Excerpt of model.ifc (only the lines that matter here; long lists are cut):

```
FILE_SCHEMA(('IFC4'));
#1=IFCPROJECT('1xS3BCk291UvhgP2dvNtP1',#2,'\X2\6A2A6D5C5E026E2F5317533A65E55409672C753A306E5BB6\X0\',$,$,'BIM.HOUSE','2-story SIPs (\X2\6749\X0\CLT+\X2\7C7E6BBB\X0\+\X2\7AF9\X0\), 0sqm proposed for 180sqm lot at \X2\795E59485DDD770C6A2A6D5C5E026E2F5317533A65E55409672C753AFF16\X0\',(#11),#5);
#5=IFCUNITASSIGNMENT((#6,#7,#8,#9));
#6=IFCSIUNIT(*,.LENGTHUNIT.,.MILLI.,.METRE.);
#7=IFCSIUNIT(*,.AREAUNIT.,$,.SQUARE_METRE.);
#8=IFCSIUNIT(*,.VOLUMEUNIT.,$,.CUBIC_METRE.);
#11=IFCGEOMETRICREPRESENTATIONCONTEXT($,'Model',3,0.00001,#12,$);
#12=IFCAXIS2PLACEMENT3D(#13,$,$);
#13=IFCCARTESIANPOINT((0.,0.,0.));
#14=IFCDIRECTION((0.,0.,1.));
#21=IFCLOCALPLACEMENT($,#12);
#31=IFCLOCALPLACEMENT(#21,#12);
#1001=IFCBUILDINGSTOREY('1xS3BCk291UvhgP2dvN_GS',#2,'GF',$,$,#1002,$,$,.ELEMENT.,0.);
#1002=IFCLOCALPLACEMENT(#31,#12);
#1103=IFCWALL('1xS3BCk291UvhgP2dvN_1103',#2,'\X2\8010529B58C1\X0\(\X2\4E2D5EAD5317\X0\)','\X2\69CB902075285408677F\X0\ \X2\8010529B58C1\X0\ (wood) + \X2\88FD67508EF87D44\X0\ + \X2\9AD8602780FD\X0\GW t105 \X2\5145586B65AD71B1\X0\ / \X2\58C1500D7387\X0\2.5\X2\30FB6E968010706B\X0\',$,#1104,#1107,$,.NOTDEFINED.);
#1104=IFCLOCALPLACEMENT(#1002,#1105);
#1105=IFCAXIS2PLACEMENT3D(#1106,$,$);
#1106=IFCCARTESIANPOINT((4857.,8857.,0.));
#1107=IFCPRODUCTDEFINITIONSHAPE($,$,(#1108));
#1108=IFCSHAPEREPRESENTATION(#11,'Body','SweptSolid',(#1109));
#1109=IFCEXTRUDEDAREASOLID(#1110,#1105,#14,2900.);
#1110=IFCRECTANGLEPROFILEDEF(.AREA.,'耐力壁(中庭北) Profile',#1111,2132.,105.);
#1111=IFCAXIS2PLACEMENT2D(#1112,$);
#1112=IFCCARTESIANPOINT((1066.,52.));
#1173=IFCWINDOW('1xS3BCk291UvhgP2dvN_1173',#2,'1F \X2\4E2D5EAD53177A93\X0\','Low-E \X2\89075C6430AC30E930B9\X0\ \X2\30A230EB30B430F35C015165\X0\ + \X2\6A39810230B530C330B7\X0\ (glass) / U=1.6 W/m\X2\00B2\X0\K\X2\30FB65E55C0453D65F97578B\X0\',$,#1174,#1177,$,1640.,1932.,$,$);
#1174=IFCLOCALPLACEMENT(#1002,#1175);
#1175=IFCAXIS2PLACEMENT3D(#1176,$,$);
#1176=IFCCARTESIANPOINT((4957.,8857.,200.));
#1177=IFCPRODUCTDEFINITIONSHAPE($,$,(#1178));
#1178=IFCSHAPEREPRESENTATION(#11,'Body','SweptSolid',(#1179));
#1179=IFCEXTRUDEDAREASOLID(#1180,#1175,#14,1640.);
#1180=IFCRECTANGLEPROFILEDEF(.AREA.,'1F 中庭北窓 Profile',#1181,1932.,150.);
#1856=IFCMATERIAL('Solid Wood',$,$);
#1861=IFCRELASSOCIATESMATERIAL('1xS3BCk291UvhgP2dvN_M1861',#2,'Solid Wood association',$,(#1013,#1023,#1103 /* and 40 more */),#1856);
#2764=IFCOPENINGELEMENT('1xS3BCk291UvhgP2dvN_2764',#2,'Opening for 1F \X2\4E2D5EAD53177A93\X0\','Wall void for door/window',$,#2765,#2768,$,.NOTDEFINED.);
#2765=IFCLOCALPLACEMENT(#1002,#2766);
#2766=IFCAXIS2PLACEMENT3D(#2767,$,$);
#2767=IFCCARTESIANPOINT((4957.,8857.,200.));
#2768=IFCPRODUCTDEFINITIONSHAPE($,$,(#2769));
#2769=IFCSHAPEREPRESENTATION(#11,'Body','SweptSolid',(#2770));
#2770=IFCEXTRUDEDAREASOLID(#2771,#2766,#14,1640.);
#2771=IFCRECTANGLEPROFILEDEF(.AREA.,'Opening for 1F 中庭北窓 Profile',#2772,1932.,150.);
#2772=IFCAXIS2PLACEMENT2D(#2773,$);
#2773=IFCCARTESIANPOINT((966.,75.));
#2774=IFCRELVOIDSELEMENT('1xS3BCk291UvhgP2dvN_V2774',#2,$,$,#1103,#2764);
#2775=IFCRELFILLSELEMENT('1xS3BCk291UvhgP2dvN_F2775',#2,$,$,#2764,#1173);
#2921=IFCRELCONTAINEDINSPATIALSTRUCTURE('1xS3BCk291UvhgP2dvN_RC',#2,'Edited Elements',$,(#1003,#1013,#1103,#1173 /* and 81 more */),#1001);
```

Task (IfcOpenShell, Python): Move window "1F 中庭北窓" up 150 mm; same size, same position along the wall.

```python
import numpy as np
import ifcopenshell
import ifcopenshell.api.geometry
import ifcopenshell.util.placement
import ifcopenshell.util.unit

model = ifcopenshell.open("model.ifc")
unit_scale = ifcopenshell.util.unit.calculate_unit_scale(model)

window = model.by_id(1173)
opening = window.FillsVoids[0].RelatingOpeningElement
dz = 0.15 / unit_scale

shift = np.array([0.0, 0.0, dz])
# The window is not placed relative to its opening, so move both.
for product in (opening, window):
    matrix = ifcopenshell.util.placement.get_local_placement(product.ObjectPlacement)
    matrix[:3, 3] += shift
    ifcopenshell.api.geometry.edit_object_placement(model, product=product, matrix=matrix, is_si=False)

print(f"moved by {dz * unit_scale:+.3f} m")

model.write("model_updated.ifc")
```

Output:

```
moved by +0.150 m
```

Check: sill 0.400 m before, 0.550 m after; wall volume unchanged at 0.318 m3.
